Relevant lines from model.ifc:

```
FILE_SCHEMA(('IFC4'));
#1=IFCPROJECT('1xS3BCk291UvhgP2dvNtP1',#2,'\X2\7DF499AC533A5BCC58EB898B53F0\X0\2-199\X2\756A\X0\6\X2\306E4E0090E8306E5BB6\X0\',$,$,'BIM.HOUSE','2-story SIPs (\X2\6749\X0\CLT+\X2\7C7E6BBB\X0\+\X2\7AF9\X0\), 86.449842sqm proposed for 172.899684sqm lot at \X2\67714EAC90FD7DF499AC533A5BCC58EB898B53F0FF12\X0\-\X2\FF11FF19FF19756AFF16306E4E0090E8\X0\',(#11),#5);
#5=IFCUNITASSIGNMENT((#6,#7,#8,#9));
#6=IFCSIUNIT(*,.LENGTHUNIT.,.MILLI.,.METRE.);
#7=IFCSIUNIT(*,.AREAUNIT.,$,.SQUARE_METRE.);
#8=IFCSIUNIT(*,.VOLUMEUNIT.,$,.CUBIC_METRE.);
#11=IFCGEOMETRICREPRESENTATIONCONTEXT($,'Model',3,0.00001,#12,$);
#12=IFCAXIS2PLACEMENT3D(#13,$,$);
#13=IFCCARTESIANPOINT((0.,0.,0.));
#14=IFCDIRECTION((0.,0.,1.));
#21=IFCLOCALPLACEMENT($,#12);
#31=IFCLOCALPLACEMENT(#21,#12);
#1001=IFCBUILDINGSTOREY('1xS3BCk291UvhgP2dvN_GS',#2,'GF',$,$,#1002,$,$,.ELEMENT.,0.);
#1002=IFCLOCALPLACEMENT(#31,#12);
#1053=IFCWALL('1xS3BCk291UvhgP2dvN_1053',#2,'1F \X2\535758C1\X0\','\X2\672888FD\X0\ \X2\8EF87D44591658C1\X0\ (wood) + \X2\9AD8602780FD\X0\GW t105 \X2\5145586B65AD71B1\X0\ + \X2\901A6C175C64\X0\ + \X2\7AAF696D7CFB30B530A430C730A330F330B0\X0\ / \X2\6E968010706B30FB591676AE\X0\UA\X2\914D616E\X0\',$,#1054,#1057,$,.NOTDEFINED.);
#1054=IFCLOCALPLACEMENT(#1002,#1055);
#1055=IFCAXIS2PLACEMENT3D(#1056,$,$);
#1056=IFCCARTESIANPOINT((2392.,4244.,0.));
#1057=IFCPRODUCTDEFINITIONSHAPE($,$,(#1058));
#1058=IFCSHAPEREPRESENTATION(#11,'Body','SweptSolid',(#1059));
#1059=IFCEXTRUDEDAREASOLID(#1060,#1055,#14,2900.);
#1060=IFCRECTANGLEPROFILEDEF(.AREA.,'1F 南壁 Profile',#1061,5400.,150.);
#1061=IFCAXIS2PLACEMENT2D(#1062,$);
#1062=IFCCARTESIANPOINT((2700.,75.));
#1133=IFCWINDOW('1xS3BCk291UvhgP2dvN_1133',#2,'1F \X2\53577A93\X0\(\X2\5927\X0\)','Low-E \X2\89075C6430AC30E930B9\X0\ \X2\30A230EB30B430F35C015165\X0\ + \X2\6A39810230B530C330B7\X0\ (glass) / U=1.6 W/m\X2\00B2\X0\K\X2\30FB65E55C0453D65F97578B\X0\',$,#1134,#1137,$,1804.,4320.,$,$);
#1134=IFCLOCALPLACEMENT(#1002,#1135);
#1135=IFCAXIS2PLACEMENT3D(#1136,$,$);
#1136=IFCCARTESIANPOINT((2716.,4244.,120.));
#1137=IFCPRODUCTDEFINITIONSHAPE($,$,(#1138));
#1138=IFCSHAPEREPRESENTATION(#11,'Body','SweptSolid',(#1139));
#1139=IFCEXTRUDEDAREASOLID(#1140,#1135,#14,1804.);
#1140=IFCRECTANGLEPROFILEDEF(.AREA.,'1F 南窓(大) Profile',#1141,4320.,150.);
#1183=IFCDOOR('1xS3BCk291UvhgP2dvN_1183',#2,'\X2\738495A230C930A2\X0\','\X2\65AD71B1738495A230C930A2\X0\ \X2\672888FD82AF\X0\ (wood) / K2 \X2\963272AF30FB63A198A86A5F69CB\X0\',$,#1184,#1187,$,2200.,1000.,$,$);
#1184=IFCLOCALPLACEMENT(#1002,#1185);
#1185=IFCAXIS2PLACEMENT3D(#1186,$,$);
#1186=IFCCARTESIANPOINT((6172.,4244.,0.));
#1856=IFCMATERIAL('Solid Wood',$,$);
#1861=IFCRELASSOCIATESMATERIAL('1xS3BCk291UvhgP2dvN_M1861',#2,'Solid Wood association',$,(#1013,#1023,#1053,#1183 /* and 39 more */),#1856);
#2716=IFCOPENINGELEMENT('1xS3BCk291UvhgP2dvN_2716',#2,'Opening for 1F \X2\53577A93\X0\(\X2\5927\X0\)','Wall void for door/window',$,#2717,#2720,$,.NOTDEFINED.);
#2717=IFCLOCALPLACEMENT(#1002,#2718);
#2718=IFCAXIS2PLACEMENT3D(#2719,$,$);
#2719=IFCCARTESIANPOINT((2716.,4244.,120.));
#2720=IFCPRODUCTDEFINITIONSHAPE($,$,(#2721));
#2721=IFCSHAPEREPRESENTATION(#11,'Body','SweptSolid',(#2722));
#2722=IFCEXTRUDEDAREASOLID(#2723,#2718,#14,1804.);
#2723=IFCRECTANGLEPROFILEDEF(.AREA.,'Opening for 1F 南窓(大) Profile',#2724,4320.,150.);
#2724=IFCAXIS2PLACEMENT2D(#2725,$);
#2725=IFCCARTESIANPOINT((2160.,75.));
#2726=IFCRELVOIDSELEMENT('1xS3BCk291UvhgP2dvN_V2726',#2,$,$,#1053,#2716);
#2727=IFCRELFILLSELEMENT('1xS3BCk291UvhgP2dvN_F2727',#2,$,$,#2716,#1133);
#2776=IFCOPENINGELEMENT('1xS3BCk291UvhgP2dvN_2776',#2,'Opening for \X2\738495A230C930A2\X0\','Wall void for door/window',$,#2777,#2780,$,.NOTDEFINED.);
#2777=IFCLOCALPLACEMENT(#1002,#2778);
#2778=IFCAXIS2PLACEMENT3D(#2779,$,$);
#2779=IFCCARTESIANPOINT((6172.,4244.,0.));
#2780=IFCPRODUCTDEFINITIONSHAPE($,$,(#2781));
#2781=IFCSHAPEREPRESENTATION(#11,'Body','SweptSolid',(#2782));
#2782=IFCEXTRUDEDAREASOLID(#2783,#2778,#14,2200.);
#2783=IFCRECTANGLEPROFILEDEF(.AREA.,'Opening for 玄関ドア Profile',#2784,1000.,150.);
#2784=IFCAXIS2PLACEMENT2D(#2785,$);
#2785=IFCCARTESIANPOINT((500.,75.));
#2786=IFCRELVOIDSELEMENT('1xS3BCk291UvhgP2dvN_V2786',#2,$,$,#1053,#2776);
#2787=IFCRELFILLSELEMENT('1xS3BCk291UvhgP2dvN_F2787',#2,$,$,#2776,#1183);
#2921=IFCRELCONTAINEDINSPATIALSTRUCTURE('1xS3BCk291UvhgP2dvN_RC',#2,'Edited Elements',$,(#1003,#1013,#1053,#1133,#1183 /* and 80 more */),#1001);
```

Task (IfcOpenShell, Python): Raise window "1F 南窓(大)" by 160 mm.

```python
import numpy as np
import ifcopenshell
import ifcopenshell.api.geometry
import ifcopenshell.util.placement
import ifcopenshell.util.unit

model = ifcopenshell.open("model.ifc")
unit_scale = ifcopenshell.util.unit.calculate_unit_scale(model)

window = model.by_guid("1xS3BCk291UvhgP2dvN_1133")
opening = window.FillsVoids[0].RelatingOpeningElement
dz = 0.16 / unit_scale

shift = np.array([0.0, 0.0, dz])
# The window is not placed relative to its opening, so move both.
for product in (opening, window):
    matrix = ifcopenshell.util.placement.get_local_placement(product.ObjectPlacement)
    matrix[:3, 3] += shift
    ifcopenshell.api.geometry.edit_object_placement(model, product=product, matrix=matrix, is_si=False)

print(f"moved by {dz * unit_scale:+.3f} m")

model.write("model_updated.ifc")
```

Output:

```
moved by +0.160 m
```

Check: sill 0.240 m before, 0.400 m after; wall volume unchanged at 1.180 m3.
